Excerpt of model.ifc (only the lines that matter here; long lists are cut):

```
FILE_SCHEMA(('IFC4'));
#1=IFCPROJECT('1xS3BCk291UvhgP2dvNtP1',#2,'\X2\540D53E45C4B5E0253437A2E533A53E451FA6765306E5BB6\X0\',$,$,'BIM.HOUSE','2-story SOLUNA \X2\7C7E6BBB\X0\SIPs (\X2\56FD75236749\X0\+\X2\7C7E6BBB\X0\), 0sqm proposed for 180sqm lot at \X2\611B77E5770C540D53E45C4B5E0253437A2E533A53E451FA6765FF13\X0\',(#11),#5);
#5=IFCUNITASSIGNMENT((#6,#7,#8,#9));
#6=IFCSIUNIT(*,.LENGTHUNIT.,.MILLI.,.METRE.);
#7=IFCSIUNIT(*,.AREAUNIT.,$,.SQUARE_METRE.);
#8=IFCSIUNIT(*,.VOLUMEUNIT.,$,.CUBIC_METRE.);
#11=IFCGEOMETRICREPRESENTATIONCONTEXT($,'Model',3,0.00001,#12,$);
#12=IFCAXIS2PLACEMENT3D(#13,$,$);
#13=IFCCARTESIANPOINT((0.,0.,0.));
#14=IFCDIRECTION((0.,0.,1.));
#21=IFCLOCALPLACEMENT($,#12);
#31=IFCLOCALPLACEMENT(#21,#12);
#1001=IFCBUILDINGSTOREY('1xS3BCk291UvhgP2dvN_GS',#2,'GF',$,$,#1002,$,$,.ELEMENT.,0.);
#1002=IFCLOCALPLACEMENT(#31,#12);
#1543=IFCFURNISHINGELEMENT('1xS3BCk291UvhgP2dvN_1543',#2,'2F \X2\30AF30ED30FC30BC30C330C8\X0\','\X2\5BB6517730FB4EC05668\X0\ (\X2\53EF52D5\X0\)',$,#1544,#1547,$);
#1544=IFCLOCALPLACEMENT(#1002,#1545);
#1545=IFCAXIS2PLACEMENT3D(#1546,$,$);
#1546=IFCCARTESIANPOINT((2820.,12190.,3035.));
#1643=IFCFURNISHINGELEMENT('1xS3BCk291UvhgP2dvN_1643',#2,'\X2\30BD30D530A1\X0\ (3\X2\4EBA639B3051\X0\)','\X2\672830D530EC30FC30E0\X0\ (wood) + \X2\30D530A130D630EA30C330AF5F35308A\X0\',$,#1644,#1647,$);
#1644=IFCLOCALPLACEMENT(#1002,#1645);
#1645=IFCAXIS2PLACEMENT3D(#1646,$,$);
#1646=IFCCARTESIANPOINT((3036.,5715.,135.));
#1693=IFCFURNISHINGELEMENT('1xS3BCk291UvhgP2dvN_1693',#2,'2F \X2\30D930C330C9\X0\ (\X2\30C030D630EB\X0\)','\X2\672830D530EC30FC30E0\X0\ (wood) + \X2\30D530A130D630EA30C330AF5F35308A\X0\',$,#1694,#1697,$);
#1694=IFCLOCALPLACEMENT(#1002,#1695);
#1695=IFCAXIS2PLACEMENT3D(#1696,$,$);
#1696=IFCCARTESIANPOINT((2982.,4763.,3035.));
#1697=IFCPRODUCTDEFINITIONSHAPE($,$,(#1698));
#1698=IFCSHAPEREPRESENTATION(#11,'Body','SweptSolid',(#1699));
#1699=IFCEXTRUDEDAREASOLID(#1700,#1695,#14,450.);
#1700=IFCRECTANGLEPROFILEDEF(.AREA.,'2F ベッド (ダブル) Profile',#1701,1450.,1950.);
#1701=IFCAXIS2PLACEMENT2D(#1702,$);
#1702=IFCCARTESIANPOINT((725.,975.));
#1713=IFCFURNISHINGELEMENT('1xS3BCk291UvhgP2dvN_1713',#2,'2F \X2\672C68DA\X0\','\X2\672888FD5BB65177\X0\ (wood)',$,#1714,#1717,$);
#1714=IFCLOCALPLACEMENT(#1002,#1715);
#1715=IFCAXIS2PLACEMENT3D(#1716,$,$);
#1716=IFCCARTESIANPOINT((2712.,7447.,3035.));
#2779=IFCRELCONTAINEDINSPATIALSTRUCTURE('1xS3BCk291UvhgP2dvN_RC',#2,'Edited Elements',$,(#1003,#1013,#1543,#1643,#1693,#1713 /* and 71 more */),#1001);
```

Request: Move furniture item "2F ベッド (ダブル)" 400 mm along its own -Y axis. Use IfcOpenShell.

```python
import ifcopenshell
import ifcopenshell.api.geometry
import ifcopenshell.util.placement

model = ifcopenshell.open("model.ifc")

item = model.by_guid("1xS3BCk291UvhgP2dvN_1693")
matrix = ifcopenshell.util.placement.get_local_placement(item.ObjectPlacement)
matrix[:3, 3] -= matrix[:3, 1] * 400.0
ifcopenshell.api.geometry.edit_object_placement(model, product=item, matrix=matrix, is_si=False)

print(ifcopenshell.util.placement.get_local_placement(item.ObjectPlacement).round(3) + 0.0)

model.write("model_updated.ifc")
```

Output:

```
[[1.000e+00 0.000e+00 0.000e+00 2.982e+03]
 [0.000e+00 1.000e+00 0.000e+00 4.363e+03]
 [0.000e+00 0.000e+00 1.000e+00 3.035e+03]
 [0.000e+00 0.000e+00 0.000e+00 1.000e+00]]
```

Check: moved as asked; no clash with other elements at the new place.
